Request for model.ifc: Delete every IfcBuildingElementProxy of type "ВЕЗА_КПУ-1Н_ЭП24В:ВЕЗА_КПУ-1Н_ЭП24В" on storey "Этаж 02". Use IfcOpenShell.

First a look at what the model holds.

```python
import ifcopenshell
import ifcopenshell.util.element

model = ifcopenshell.open("model.ifc")
print(model.schema)
storey = next(s for s in model.by_type("IfcBuildingStorey") if s.Name == "Этаж 02")
proxies = [e for e in ifcopenshell.util.element.get_decomposition(storey) if e.is_a("IfcBuildingElementProxy")]
seen = {}
for e in proxies:
    element_type = ifcopenshell.util.element.get_type(e)
    name = element_type.Name if element_type not in (None, e) else None
    seen[name] = seen.get(name, 0) + 1
for name, count in sorted(seen.items(), key=str):
    print(count, "x", name)
```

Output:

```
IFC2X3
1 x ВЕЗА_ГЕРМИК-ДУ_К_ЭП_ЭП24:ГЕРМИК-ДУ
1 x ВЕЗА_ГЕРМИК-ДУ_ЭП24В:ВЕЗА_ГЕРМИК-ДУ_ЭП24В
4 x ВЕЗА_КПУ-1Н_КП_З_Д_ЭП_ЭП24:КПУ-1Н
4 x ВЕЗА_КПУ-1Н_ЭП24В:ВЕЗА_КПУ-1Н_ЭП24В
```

```python
import ifcopenshell
import ifcopenshell.api.root
import ifcopenshell.util.element

model = ifcopenshell.open("model.ifc")

storey = next(s for s in model.by_type("IfcBuildingStorey") if s.Name == "Этаж 02")
proxies = [e for e in ifcopenshell.util.element.get_decomposition(storey) if e.is_a("IfcBuildingElementProxy")]
targets = [e for e in proxies if (t := ifcopenshell.util.element.get_type(e)) not in (None, e) and t.Name == "ВЕЗА_КПУ-1Н_ЭП24В:ВЕЗА_КПУ-1Н_ЭП24В"]

for e in targets:
    ifcopenshell.api.root.remove_product(model, product=e)
print(len(targets), "removed")

model.write("model_updated.ifc")
```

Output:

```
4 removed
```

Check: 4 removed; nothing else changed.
